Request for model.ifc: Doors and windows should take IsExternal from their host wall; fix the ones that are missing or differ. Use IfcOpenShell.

First a look at what the model holds.

```python
import ifcopenshell
import ifcopenshell.util.element

model = ifcopenshell.open("model.ifc")
print(model.schema)
seen = {}
for e in model.by_type("IfcDoor") + model.by_type("IfcWindow"):
    if not e.FillsVoids:
        continue
    host = e.FillsVoids[0].RelatingOpeningElement.VoidsElements[0].RelatingBuildingElement
    own = ifcopenshell.util.element.get_pset(e, f"Pset_{e.is_a()[3:].removesuffix('StandardCase')}Common", "IsExternal")
    wall = ifcopenshell.util.element.get_pset(host, "Pset_WallCommon", "IsExternal")
    seen[e.is_a(), own, wall] = seen.get((e.is_a(), own, wall), 0) + 1
for (cls, own, wall), count in sorted(seen.items(), key=str):
    print(count, cls, "IsExternal:", own, "| host wall:", wall)
```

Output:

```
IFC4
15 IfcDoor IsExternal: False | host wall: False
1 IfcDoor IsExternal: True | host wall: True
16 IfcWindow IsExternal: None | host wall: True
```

```python
import ifcopenshell
import ifcopenshell.api.pset
import ifcopenshell.util.element

model = ifcopenshell.open("model.ifc")

count = 0
for ifc_class, pset_name in (("IfcDoor", "Pset_DoorCommon"), ("IfcWindow", "Pset_WindowCommon")):
    for e in model.by_type(ifc_class):
        if not e.FillsVoids:
            continue
        host = e.FillsVoids[0].RelatingOpeningElement.VoidsElements[0].RelatingBuildingElement
        external = ifcopenshell.util.element.get_pset(host, "Pset_WallCommon", "IsExternal")
        if external is None or ifcopenshell.util.element.get_pset(e, pset_name, "IsExternal") == external:
            continue
        pset = ifcopenshell.api.pset.add_pset(model, product=e, name=pset_name)
        ifcopenshell.api.pset.edit_pset(model, pset=pset, properties={"IsExternal": external})
        count += 1

print(count, "updated")

model.write("model_updated.ifc")
```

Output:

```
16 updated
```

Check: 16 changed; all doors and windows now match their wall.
